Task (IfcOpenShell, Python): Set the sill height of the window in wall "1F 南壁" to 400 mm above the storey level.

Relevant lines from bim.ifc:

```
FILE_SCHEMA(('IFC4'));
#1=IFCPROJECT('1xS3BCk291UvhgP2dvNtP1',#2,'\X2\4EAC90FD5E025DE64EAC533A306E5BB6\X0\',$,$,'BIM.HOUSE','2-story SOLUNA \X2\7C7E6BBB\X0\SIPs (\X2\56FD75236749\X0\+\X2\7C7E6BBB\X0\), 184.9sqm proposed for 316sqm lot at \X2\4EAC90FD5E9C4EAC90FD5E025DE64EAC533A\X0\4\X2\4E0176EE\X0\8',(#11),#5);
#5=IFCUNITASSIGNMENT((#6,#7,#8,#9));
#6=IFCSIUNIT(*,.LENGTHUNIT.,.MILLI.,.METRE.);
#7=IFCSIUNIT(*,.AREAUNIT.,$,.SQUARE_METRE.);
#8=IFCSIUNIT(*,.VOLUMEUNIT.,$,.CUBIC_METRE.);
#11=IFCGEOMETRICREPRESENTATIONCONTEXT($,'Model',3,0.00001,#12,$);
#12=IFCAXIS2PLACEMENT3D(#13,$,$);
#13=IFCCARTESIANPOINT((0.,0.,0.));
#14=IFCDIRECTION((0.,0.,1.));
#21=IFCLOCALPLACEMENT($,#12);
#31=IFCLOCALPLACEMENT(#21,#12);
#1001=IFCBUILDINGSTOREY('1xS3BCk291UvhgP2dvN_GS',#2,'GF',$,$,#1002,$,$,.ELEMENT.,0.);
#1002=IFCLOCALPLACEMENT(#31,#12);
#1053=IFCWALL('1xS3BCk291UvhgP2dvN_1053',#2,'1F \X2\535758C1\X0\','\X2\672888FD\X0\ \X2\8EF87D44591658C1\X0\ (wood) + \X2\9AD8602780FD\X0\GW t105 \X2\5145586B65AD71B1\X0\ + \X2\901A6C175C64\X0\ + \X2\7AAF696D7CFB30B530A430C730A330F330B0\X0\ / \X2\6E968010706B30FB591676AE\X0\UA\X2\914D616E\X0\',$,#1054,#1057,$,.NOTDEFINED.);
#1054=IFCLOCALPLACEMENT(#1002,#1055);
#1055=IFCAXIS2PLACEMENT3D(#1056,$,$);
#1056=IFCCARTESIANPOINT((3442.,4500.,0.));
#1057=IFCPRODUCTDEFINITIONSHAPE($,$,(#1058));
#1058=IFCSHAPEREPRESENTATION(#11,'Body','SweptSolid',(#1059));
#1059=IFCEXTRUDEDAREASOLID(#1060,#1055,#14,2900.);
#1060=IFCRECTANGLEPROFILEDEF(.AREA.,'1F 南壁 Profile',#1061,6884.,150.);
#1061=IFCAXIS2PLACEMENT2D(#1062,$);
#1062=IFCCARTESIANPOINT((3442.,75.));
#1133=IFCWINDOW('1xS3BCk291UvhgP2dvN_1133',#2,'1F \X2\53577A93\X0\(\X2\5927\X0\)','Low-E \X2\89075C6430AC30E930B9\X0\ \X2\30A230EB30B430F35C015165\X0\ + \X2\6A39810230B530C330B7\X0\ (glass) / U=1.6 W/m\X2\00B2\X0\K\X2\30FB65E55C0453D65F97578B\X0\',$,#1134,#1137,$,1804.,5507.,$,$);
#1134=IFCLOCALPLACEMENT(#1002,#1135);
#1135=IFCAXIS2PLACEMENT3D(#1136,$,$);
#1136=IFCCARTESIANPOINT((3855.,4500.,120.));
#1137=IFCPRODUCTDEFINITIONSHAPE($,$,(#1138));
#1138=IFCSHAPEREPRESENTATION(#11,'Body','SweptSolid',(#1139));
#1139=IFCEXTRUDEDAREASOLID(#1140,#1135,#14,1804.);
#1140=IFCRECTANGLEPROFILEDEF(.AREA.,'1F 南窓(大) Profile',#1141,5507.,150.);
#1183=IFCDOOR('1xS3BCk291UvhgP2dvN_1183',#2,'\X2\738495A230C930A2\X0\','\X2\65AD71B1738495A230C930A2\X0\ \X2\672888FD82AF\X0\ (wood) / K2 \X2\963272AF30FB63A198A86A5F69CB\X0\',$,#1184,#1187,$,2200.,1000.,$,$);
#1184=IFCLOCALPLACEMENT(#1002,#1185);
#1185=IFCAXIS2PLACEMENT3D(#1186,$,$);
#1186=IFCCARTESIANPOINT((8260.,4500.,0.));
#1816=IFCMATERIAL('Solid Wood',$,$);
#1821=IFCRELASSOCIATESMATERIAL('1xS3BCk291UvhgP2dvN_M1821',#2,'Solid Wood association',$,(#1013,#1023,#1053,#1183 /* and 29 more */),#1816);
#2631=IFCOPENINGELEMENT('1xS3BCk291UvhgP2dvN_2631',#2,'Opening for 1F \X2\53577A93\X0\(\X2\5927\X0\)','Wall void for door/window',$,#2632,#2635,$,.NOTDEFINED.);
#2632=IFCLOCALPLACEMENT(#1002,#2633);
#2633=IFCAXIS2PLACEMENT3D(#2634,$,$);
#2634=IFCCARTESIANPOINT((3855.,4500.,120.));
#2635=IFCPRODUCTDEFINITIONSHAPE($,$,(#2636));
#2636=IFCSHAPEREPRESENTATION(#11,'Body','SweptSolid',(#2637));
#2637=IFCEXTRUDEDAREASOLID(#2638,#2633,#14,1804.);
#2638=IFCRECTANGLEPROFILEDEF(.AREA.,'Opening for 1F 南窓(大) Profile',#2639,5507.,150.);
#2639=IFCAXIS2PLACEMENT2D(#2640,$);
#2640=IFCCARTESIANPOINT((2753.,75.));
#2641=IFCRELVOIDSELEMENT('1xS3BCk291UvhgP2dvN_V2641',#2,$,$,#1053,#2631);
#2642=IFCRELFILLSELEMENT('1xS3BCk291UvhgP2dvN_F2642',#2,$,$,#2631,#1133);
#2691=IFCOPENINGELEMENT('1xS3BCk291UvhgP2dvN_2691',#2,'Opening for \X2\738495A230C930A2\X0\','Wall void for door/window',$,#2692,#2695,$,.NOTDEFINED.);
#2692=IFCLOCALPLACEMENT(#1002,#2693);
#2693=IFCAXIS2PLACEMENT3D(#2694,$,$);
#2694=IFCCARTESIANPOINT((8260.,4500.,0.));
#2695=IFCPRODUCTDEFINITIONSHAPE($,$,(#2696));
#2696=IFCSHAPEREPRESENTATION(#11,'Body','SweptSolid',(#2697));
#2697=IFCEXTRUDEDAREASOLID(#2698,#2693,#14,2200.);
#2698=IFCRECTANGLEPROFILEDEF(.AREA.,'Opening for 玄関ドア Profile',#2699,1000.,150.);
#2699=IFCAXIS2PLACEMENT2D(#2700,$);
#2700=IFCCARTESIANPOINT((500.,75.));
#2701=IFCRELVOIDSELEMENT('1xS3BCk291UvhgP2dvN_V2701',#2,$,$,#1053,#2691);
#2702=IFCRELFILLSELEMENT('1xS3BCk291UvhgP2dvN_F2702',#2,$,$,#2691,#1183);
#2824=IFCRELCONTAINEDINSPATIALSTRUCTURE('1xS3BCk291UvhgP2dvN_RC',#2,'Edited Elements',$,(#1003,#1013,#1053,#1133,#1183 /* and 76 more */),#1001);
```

```python
import numpy as np
import ifcopenshell
import ifcopenshell.api.geometry
import ifcopenshell.geom
import ifcopenshell.util.element
import ifcopenshell.util.placement
import ifcopenshell.util.shape
import ifcopenshell.util.unit

model = ifcopenshell.open("bim.ifc")
unit_scale = ifcopenshell.util.unit.calculate_unit_scale(model)

window = model.by_guid("1xS3BCk291UvhgP2dvN_1133")
opening = window.FillsVoids[0].RelatingOpeningElement
storey = ifcopenshell.util.element.get_container(window, ifc_class="IfcBuildingStorey")
level = ifcopenshell.util.placement.get_local_placement(storey.ObjectPlacement)[2, 3]

# The opening's origin need not be at the sill, so measure its lowest point.
shape = ifcopenshell.geom.create_shape(ifcopenshell.geom.settings(), opening)
bottom = ifcopenshell.util.shape.get_shape_bottom_elevation(shape, shape.geometry) / unit_scale
dz = level + 400.0 - bottom

shift = np.array([0.0, 0.0, dz])
# The window is not placed relative to its opening, so move both.
for product in (opening, window):
    matrix = ifcopenshell.util.placement.get_local_placement(product.ObjectPlacement)
    matrix[:3, 3] += shift
    ifcopenshell.api.geometry.edit_object_placement(model, product=product, matrix=matrix, is_si=False)

print(f"moved by {dz * unit_scale:+.3f} m")

model.write("bim_rev.ifc")
```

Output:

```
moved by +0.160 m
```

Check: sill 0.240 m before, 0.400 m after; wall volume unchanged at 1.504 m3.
